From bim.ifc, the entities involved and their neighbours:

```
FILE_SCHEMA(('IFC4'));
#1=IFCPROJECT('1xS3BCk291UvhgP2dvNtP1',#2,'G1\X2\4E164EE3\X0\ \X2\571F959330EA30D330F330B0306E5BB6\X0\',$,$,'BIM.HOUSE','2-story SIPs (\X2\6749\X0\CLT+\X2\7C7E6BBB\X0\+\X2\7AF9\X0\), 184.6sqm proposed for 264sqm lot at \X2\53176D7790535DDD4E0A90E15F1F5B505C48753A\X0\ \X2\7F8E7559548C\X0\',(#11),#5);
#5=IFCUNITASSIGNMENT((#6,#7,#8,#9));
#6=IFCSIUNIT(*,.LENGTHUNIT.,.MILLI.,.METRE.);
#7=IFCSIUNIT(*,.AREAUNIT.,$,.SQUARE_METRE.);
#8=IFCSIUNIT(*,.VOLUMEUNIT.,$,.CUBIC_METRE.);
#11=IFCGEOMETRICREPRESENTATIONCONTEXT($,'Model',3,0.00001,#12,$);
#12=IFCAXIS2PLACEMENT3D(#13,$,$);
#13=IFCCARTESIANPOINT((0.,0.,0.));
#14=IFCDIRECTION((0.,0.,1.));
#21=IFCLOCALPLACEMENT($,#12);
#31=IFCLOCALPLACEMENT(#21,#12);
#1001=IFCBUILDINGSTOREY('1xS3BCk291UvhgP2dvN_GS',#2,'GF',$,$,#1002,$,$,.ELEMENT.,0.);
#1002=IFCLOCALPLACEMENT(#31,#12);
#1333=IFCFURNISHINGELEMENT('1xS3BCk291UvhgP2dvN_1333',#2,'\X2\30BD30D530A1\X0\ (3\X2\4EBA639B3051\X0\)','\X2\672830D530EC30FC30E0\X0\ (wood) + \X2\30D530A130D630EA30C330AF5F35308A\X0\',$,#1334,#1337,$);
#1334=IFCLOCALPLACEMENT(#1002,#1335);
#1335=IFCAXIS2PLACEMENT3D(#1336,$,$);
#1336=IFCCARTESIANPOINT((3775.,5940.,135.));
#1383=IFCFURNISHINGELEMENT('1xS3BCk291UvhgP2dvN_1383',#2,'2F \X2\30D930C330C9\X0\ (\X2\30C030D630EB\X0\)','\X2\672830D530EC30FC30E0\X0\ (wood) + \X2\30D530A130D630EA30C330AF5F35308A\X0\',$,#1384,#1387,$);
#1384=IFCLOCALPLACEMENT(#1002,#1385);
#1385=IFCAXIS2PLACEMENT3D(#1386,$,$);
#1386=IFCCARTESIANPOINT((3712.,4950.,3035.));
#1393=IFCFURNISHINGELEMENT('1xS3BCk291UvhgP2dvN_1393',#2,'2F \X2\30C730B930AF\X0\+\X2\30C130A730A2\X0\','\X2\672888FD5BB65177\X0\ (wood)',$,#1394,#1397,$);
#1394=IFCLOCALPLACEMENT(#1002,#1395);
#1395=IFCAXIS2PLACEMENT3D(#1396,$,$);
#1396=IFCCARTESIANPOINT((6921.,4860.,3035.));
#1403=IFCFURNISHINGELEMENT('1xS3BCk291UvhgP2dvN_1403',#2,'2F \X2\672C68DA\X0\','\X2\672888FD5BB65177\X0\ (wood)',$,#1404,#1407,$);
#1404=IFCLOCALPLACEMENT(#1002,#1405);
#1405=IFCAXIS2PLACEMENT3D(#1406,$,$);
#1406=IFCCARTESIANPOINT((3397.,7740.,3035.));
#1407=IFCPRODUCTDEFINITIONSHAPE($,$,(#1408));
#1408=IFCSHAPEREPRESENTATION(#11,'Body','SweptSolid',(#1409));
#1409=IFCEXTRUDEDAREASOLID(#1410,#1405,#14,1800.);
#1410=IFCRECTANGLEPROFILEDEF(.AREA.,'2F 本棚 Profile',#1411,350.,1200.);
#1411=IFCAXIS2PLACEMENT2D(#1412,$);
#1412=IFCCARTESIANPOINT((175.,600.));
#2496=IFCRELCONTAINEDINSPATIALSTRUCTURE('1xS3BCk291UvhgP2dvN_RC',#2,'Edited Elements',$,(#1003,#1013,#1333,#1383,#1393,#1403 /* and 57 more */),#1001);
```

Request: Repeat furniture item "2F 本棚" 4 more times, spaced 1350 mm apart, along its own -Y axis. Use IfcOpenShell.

```python
import ifcopenshell
import ifcopenshell.api.geometry
import ifcopenshell.api.root
import ifcopenshell.util.element
import ifcopenshell.util.placement
import ifcopenshell.util.unit

model = ifcopenshell.open("bim.ifc")
unit_scale = ifcopenshell.util.unit.calculate_unit_scale(model)


def reuse_history(source, copy):
    """copy_class also copies each property set's owner history, people and application; keep the originals."""
    for rel in copy.IsDefinedBy:
        if rel.is_a("IfcRelDefinesByProperties") and (history := rel.RelatingPropertyDefinition.OwnerHistory):
            rel.RelatingPropertyDefinition.OwnerHistory = source.OwnerHistory
            ifcopenshell.util.element.remove_deep2(model, history)


source = model.by_guid("1xS3BCk291UvhgP2dvN_1403")
base = ifcopenshell.util.placement.get_local_placement(source.ObjectPlacement)
step = -base[:3, 1] * 1.35 / unit_scale

for i in range(1, 5):
    copy = ifcopenshell.api.root.copy_class(model, product=source)
    copy.Representation = ifcopenshell.util.element.copy_deep(
        model, source.Representation, exclude=["IfcGeometricRepresentationContext", "IfcRepresentationMap"]
    )
    reuse_history(source, copy)
    matrix = base.copy()
    matrix[:3, 3] += i * step
    print("added at", matrix[:3, 3].round(3) + 0.0)
    ifcopenshell.api.geometry.edit_object_placement(model, product=copy, matrix=matrix, is_si=False)

model.write("bim-out.ifc")
```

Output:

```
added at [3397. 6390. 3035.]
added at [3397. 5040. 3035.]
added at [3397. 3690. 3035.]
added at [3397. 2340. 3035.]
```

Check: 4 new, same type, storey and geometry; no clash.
